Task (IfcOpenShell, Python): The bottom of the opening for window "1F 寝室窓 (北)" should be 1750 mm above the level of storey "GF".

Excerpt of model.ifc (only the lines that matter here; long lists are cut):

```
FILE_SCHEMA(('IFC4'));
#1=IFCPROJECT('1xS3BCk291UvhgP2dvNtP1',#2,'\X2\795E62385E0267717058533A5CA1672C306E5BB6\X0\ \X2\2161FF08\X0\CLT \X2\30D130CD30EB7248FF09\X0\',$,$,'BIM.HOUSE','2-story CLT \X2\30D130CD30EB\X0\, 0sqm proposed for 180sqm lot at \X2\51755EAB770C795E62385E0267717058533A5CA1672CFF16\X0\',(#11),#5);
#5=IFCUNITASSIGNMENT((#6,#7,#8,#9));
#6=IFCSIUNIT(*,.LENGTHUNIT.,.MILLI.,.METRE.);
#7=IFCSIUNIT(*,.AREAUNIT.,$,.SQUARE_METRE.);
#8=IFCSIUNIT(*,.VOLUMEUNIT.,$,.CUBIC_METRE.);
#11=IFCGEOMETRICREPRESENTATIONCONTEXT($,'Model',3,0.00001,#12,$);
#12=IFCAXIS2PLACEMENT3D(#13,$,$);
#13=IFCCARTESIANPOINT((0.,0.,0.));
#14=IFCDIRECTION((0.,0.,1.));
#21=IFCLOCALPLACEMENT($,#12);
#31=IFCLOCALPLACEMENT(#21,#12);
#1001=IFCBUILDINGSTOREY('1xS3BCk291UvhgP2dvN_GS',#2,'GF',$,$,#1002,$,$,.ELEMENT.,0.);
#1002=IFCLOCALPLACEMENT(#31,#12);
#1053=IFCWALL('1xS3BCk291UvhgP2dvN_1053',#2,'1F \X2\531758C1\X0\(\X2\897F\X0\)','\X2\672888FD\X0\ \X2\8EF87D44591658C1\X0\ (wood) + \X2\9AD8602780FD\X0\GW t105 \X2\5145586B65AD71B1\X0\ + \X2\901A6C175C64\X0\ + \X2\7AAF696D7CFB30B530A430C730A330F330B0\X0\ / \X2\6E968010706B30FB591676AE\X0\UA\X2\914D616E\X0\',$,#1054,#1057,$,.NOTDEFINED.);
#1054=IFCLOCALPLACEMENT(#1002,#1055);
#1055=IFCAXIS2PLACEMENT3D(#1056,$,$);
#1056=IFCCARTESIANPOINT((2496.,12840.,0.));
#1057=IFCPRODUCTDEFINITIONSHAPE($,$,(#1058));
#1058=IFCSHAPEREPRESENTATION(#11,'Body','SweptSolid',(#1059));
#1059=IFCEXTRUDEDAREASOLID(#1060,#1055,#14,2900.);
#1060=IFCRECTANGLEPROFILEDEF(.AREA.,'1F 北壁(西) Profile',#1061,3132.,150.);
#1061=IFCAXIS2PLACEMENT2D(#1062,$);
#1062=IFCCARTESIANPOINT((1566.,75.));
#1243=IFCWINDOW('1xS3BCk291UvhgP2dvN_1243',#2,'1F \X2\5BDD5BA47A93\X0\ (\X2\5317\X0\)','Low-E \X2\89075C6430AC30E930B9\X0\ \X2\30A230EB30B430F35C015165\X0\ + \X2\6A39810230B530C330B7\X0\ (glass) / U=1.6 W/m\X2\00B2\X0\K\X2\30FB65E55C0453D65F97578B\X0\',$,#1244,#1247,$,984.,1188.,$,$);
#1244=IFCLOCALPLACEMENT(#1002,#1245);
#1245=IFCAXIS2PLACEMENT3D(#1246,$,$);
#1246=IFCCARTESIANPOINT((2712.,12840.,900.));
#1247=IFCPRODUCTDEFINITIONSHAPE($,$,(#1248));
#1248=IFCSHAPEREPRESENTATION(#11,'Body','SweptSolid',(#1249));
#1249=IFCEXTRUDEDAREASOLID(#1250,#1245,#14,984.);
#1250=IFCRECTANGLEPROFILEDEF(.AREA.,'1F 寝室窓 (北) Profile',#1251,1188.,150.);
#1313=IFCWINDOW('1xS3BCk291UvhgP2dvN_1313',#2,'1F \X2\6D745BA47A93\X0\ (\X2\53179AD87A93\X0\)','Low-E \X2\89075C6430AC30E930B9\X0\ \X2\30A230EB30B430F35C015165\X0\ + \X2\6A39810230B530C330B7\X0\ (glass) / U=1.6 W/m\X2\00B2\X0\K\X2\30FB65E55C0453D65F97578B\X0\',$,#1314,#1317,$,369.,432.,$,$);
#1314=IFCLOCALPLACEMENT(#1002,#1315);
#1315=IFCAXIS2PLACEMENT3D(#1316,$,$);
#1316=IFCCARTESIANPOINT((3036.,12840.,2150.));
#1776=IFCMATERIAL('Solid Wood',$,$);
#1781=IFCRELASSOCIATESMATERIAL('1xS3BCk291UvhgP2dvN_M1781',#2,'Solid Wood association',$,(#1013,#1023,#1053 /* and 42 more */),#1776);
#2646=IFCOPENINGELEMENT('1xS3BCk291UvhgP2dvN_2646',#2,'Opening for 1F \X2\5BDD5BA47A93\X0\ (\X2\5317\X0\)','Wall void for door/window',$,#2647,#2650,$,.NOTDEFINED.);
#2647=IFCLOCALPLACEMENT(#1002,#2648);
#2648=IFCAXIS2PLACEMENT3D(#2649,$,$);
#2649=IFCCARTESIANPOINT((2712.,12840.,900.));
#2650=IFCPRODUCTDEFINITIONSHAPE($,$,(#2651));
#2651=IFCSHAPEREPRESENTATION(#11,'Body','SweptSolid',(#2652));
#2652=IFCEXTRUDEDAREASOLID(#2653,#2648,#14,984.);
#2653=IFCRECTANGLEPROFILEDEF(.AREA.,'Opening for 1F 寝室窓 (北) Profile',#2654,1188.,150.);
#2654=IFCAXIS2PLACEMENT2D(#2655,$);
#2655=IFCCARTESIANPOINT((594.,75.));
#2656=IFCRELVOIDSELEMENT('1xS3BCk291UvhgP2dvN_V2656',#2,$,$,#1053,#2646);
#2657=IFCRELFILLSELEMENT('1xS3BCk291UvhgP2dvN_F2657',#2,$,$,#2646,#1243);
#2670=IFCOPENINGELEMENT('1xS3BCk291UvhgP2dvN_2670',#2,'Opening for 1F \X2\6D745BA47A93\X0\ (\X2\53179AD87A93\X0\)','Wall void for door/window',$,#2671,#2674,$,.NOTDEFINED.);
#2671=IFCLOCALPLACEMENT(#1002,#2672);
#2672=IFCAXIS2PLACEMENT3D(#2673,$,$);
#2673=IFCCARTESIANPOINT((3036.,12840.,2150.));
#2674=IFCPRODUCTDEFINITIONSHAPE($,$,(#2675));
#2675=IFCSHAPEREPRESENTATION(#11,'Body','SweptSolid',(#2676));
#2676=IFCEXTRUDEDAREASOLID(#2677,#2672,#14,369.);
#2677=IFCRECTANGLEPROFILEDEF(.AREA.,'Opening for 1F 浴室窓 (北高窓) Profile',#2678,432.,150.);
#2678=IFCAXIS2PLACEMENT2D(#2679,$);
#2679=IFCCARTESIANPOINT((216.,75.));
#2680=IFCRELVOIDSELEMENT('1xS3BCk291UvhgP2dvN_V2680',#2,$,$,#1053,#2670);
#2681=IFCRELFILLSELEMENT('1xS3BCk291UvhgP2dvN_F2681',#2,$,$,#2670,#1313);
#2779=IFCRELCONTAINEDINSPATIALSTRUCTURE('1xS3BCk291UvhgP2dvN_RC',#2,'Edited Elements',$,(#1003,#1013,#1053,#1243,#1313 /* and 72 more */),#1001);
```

```python
import numpy as np
import ifcopenshell
import ifcopenshell.api.geometry
import ifcopenshell.geom
import ifcopenshell.util.element
import ifcopenshell.util.placement
import ifcopenshell.util.shape
import ifcopenshell.util.unit

model = ifcopenshell.open("model.ifc")
unit_scale = ifcopenshell.util.unit.calculate_unit_scale(model)

window = model.by_guid("1xS3BCk291UvhgP2dvN_1243")
opening = window.FillsVoids[0].RelatingOpeningElement
storey = ifcopenshell.util.element.get_container(window, ifc_class="IfcBuildingStorey")
level = ifcopenshell.util.placement.get_local_placement(storey.ObjectPlacement)[2, 3]

# The opening's origin need not be at the sill, so measure its lowest point.
shape = ifcopenshell.geom.create_shape(ifcopenshell.geom.settings(), opening)
bottom = ifcopenshell.util.shape.get_shape_bottom_elevation(shape, shape.geometry) / unit_scale
dz = level + 1750.0 - bottom

shift = np.array([0.0, 0.0, dz])
# The window is not placed relative to its opening, so move both.
for product in (opening, window):
    matrix = ifcopenshell.util.placement.get_local_placement(product.ObjectPlacement)
    matrix[:3, 3] += shift
    ifcopenshell.api.geometry.edit_object_placement(model, product=product, matrix=matrix, is_si=False)

print(f"moved by {dz * unit_scale:+.3f} m")

model.write("model_rev.ifc")
```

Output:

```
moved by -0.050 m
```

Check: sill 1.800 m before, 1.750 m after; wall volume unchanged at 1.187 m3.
